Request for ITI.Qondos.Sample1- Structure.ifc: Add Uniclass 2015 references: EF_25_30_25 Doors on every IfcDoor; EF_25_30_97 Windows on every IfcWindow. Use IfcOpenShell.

First a look at what the model holds.

```python
import ifcopenshell

model = ifcopenshell.open("ITI.Qondos.Sample1- Structure.ifc")
print(model.schema)
print("classifications:", [c.Name for c in model.by_type("IfcClassification")])
for ifc_class in ("IfcDoor", "IfcRoof", "IfcStair", "IfcWall", "IfcWindow"):
    print(ifc_class, len(model.by_type(ifc_class)))
```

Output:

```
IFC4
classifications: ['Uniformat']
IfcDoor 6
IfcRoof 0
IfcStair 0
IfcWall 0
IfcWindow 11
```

```python
import ifcopenshell
import ifcopenshell.api.classification

model = ifcopenshell.open("ITI.Qondos.Sample1- Structure.ifc")

system = ifcopenshell.api.classification.add_classification(model, classification="Uniclass 2015")

codes = {
    "IfcDoor": ("EF_25_30_25", "Doors"),
    "IfcWindow": ("EF_25_30_97", "Windows"),
}
for ifc_class, (code, name) in codes.items():
    products = model.by_type(ifc_class)
    ifcopenshell.api.classification.add_reference(
        model, products=products, classification=system, identification=code, name=name
    )
    print(code, len(products))

model.write("ITI.Qondos.Sample1- Structure_edited.ifc")
```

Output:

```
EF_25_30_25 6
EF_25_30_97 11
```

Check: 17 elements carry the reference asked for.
